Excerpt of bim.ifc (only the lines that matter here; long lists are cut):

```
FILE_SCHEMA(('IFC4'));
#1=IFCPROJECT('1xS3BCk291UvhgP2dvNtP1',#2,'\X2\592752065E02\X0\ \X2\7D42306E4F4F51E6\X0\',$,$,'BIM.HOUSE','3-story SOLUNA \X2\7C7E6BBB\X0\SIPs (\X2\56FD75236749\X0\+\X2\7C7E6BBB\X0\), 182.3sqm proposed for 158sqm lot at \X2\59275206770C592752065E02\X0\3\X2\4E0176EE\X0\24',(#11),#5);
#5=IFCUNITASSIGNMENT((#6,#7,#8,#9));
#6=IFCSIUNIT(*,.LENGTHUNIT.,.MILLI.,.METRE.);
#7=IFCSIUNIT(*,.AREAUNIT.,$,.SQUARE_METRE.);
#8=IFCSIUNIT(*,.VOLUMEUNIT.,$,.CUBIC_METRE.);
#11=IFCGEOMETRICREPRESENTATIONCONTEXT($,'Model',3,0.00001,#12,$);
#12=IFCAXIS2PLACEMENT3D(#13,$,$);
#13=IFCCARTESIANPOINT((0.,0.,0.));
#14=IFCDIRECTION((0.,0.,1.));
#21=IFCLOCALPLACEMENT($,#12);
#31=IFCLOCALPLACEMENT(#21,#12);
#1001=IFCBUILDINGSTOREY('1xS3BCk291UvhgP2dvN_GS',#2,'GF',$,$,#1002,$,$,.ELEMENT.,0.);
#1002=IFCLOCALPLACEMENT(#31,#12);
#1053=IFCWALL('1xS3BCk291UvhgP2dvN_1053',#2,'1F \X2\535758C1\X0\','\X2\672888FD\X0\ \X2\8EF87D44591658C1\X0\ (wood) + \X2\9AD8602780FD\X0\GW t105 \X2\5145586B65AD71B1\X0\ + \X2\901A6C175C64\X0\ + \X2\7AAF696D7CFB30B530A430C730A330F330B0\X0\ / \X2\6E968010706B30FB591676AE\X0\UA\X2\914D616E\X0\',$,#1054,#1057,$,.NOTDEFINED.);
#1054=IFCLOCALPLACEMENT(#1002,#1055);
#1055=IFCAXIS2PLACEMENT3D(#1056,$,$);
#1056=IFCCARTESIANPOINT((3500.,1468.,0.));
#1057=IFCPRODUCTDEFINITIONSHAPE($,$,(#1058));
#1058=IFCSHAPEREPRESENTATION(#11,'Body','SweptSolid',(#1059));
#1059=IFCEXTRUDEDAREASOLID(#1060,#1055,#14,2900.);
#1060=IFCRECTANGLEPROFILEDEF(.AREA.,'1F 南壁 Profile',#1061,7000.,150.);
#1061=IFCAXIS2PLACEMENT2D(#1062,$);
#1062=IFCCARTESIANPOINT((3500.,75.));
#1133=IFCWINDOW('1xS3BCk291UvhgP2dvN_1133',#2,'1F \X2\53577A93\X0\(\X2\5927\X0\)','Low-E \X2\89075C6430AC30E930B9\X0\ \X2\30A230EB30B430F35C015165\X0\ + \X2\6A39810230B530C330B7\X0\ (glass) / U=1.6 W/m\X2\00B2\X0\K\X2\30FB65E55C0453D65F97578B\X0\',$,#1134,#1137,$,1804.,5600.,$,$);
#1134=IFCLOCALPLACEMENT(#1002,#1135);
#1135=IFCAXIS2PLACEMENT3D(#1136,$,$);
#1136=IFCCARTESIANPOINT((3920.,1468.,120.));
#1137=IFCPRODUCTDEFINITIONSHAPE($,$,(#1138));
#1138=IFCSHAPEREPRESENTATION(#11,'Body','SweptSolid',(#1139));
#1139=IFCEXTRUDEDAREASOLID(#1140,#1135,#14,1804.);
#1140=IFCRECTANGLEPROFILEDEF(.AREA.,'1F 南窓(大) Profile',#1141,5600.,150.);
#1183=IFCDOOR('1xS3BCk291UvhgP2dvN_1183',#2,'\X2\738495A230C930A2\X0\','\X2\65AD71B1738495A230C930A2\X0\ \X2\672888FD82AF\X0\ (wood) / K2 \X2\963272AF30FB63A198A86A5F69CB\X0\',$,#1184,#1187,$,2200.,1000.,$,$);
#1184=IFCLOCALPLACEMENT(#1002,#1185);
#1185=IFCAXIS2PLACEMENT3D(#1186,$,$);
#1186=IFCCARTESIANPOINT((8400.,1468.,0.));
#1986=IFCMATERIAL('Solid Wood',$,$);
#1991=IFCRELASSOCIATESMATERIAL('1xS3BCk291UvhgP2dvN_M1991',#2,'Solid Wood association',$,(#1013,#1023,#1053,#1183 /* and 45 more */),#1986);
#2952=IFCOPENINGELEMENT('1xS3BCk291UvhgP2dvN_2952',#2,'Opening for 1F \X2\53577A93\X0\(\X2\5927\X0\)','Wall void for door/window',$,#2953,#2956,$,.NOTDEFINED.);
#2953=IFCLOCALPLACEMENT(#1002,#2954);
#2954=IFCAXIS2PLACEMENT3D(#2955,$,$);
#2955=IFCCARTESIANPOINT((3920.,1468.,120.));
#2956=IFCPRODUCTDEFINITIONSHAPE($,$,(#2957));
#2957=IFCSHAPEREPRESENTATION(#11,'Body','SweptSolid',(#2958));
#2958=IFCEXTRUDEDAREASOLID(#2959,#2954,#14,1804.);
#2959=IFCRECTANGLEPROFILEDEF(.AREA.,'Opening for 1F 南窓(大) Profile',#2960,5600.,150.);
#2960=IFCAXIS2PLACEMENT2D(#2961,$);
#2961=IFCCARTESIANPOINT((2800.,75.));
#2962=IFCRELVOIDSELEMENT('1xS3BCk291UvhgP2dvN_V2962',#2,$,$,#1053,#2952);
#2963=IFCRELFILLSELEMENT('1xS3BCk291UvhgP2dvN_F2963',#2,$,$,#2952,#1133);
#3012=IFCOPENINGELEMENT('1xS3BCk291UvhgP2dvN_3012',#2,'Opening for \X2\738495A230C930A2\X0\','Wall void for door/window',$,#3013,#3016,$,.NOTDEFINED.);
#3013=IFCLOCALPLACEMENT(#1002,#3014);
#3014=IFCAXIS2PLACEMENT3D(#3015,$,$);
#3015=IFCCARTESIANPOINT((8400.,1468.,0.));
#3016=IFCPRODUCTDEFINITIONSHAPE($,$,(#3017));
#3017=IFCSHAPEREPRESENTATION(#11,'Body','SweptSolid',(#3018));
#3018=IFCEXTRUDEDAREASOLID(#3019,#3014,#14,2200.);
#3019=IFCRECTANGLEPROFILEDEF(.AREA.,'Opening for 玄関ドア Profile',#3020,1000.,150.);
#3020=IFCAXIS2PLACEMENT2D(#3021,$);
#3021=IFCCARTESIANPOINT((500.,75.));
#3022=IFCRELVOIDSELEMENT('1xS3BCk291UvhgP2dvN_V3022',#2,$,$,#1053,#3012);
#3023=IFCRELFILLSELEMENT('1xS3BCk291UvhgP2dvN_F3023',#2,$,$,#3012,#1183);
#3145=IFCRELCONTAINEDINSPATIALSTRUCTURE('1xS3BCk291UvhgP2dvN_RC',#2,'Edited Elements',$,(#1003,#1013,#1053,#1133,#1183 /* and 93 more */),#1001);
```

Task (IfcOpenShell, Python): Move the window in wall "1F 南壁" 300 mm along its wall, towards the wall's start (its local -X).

```python
import ifcopenshell
import ifcopenshell.api.geometry
import ifcopenshell.util.placement

model = ifcopenshell.open("bim.ifc")

window = model.by_guid("1xS3BCk291UvhgP2dvN_1133")
opening = window.FillsVoids[0].RelatingOpeningElement
wall = opening.VoidsElements[0].RelatingBuildingElement

wall_matrix = ifcopenshell.util.placement.get_local_placement(wall.ObjectPlacement)
shift = wall_matrix[:3, 0] * -300.0
before = ifcopenshell.util.placement.get_local_placement(window.ObjectPlacement)[:3, 3].copy()

# The window is not placed relative to its opening, so move both.
for product in (opening, window):
    matrix = ifcopenshell.util.placement.get_local_placement(product.ObjectPlacement)
    matrix[:3, 3] += shift
    ifcopenshell.api.geometry.edit_object_placement(model, product=product, matrix=matrix, is_si=False)

after = ifcopenshell.util.placement.get_local_placement(window.ObjectPlacement)[:3, 3]
print("window moved by", (after - before).round(3) + 0.0)

model.write("bim_v2.ifc")
```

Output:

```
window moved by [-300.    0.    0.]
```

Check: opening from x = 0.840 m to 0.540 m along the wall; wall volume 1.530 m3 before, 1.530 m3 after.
